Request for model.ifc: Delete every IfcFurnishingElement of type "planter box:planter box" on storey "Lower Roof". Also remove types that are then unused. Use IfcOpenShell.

First a look at what the model holds.

```python
import ifcopenshell
import ifcopenshell.util.element

model = ifcopenshell.open("model.ifc")
print(model.schema)
storey = next(s for s in model.by_type("IfcBuildingStorey") if s.Name == "Lower Roof")
furniture = [e for e in ifcopenshell.util.element.get_decomposition(storey) if e.is_a("IfcFurnishingElement")]
seen = {}
for e in furniture:
    element_type = ifcopenshell.util.element.get_type(e)
    name = element_type.Name if element_type not in (None, e) else None
    seen[name] = seen.get(name, 0) + 1
for name, count in sorted(seen.items(), key=str):
    print(count, "x", name)
```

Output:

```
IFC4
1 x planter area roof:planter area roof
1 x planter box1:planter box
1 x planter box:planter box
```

```python
import ifcopenshell
import ifcopenshell.api.root
import ifcopenshell.util.element

model = ifcopenshell.open("model.ifc")

storey = next(s for s in model.by_type("IfcBuildingStorey") if s.Name == "Lower Roof")
furniture = [e for e in ifcopenshell.util.element.get_decomposition(storey) if e.is_a("IfcFurnishingElement")]
targets = [e for e in furniture if (t := ifcopenshell.util.element.get_type(e)) not in (None, e) and t.Name == "planter box:planter box"]
types = {ifcopenshell.util.element.get_type(e) for e in targets} - {None, *targets}

for e in targets:
    ifcopenshell.api.root.remove_product(model, product=e)
print(len(targets), "removed")

unused = [t for t in types if not ifcopenshell.util.element.get_types(t)]
for t in unused:
    ifcopenshell.api.root.remove_product(model, product=t)
print(len(unused), "unused types removed")

model.write("model_rev.ifc")
```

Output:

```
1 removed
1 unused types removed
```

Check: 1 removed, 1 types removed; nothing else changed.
